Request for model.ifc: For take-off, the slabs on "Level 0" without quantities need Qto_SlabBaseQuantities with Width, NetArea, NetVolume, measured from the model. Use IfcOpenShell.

First a look at what the model holds.

```python
import ifcopenshell
import ifcopenshell.util.element
import ifcopenshell.util.unit

model = ifcopenshell.open("model.ifc")
print(model.schema)
for unit_type in ("LENGTHUNIT", "AREAUNIT", "VOLUMEUNIT"):
    print(unit_type, ifcopenshell.util.unit.calculate_unit_scale(model, unit_type))
storey = next(s for s in model.by_type("IfcBuildingStorey") if s.Name == "Level 0")
slabs = [e for e in ifcopenshell.util.element.get_decomposition(storey) if e.is_a("IfcSlab")]
for e in sorted(slabs, key=lambda e: e.id()):
    print(e.id(), e.is_a(), e.Name, list(ifcopenshell.util.element.get_psets(e, qtos_only=True)), sep=" | ")
```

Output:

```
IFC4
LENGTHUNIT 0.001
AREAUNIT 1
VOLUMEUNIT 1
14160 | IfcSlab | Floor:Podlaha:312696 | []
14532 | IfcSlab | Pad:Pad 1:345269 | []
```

```python
import ifcopenshell
import ifcopenshell.api.pset
import ifcopenshell.geom
import ifcopenshell.util.element
import ifcopenshell.util.shape
import ifcopenshell.util.unit

model = ifcopenshell.open("model.ifc")
unit_scale = ifcopenshell.util.unit.calculate_unit_scale(model)
area_scale = ifcopenshell.util.unit.calculate_unit_scale(model, "AREAUNIT")
volume_scale = ifcopenshell.util.unit.calculate_unit_scale(model, "VOLUMEUNIT")
settings = ifcopenshell.geom.settings()

storey = next(s for s in model.by_type("IfcBuildingStorey") if s.Name == "Level 0")
slabs = [e for e in ifcopenshell.util.element.get_decomposition(storey) if e.is_a("IfcSlab")]

for e in sorted(slabs, key=lambda e: e.id()):
    if ifcopenshell.util.element.get_psets(e, qtos_only=True, should_inherit=False):
        continue
    # Geometry comes back in metres, in the element's own axes.
    shape = ifcopenshell.geom.create_shape(settings, e)
    values = {
        "Width": ifcopenshell.util.shape.get_z(shape.geometry) / unit_scale,
        "NetArea": ifcopenshell.util.shape.get_footprint_area(shape.geometry) / area_scale,
        "NetVolume": ifcopenshell.util.shape.get_volume(shape.geometry) / volume_scale,
    }
    qto = ifcopenshell.api.pset.add_qto(model, product=e, name="Qto_SlabBaseQuantities")
    ifcopenshell.api.pset.edit_qto(model, qto=qto, properties=values)
    print(e.id(), {k: round(v, 3) for k, v in values.items()})

model.write("model_edited.ifc")
```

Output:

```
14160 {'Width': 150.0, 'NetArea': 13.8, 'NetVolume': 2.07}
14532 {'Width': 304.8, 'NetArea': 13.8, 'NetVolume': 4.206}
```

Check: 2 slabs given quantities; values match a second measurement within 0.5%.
